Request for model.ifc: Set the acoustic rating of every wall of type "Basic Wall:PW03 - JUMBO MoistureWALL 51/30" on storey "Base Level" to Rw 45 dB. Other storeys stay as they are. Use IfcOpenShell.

First a look at what the model holds.

```python
import ifcopenshell
import ifcopenshell.util.element

model = ifcopenshell.open("model.ifc")
print(model.schema)
storey = next(s for s in model.by_type("IfcBuildingStorey") if s.Name == "Base Level")
walls = [e for e in ifcopenshell.util.element.get_decomposition(storey) if e.is_a("IfcWall")]
seen = {}
for e in walls:
    element_type = ifcopenshell.util.element.get_type(e)
    key = (element_type.Name if element_type != e and element_type else None, ifcopenshell.util.element.get_pset(e, "Pset_WallCommon", "AcousticRating"))
    seen[key] = seen.get(key, 0) + 1
for (name, value), count in sorted(seen.items(), key=str):
    print(count, "x", name, "|", value)
```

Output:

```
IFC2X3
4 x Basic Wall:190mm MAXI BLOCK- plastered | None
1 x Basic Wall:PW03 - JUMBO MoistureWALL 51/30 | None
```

```python
import ifcopenshell
import ifcopenshell.api.pset
import ifcopenshell.util.element

model = ifcopenshell.open("model.ifc")

storey = next(s for s in model.by_type("IfcBuildingStorey") if s.Name == "Base Level")
walls = [e for e in ifcopenshell.util.element.get_decomposition(storey) if e.is_a("IfcWall")]

count = 0
for e in walls:
    element_type = ifcopenshell.util.element.get_type(e)
    if element_type in (None, e) or element_type.Name != "Basic Wall:PW03 - JUMBO MoistureWALL 51/30":
        continue
    # add_pset returns the element's existing set when there is one.
    pset = ifcopenshell.api.pset.add_pset(model, product=e, name="Pset_WallCommon")
    ifcopenshell.api.pset.edit_pset(model, pset=pset, properties={"AcousticRating": "Rw 45 dB"})
    count += 1

print(count, "walls updated")

model.write("model_rev.ifc")
```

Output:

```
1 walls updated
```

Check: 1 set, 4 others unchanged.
